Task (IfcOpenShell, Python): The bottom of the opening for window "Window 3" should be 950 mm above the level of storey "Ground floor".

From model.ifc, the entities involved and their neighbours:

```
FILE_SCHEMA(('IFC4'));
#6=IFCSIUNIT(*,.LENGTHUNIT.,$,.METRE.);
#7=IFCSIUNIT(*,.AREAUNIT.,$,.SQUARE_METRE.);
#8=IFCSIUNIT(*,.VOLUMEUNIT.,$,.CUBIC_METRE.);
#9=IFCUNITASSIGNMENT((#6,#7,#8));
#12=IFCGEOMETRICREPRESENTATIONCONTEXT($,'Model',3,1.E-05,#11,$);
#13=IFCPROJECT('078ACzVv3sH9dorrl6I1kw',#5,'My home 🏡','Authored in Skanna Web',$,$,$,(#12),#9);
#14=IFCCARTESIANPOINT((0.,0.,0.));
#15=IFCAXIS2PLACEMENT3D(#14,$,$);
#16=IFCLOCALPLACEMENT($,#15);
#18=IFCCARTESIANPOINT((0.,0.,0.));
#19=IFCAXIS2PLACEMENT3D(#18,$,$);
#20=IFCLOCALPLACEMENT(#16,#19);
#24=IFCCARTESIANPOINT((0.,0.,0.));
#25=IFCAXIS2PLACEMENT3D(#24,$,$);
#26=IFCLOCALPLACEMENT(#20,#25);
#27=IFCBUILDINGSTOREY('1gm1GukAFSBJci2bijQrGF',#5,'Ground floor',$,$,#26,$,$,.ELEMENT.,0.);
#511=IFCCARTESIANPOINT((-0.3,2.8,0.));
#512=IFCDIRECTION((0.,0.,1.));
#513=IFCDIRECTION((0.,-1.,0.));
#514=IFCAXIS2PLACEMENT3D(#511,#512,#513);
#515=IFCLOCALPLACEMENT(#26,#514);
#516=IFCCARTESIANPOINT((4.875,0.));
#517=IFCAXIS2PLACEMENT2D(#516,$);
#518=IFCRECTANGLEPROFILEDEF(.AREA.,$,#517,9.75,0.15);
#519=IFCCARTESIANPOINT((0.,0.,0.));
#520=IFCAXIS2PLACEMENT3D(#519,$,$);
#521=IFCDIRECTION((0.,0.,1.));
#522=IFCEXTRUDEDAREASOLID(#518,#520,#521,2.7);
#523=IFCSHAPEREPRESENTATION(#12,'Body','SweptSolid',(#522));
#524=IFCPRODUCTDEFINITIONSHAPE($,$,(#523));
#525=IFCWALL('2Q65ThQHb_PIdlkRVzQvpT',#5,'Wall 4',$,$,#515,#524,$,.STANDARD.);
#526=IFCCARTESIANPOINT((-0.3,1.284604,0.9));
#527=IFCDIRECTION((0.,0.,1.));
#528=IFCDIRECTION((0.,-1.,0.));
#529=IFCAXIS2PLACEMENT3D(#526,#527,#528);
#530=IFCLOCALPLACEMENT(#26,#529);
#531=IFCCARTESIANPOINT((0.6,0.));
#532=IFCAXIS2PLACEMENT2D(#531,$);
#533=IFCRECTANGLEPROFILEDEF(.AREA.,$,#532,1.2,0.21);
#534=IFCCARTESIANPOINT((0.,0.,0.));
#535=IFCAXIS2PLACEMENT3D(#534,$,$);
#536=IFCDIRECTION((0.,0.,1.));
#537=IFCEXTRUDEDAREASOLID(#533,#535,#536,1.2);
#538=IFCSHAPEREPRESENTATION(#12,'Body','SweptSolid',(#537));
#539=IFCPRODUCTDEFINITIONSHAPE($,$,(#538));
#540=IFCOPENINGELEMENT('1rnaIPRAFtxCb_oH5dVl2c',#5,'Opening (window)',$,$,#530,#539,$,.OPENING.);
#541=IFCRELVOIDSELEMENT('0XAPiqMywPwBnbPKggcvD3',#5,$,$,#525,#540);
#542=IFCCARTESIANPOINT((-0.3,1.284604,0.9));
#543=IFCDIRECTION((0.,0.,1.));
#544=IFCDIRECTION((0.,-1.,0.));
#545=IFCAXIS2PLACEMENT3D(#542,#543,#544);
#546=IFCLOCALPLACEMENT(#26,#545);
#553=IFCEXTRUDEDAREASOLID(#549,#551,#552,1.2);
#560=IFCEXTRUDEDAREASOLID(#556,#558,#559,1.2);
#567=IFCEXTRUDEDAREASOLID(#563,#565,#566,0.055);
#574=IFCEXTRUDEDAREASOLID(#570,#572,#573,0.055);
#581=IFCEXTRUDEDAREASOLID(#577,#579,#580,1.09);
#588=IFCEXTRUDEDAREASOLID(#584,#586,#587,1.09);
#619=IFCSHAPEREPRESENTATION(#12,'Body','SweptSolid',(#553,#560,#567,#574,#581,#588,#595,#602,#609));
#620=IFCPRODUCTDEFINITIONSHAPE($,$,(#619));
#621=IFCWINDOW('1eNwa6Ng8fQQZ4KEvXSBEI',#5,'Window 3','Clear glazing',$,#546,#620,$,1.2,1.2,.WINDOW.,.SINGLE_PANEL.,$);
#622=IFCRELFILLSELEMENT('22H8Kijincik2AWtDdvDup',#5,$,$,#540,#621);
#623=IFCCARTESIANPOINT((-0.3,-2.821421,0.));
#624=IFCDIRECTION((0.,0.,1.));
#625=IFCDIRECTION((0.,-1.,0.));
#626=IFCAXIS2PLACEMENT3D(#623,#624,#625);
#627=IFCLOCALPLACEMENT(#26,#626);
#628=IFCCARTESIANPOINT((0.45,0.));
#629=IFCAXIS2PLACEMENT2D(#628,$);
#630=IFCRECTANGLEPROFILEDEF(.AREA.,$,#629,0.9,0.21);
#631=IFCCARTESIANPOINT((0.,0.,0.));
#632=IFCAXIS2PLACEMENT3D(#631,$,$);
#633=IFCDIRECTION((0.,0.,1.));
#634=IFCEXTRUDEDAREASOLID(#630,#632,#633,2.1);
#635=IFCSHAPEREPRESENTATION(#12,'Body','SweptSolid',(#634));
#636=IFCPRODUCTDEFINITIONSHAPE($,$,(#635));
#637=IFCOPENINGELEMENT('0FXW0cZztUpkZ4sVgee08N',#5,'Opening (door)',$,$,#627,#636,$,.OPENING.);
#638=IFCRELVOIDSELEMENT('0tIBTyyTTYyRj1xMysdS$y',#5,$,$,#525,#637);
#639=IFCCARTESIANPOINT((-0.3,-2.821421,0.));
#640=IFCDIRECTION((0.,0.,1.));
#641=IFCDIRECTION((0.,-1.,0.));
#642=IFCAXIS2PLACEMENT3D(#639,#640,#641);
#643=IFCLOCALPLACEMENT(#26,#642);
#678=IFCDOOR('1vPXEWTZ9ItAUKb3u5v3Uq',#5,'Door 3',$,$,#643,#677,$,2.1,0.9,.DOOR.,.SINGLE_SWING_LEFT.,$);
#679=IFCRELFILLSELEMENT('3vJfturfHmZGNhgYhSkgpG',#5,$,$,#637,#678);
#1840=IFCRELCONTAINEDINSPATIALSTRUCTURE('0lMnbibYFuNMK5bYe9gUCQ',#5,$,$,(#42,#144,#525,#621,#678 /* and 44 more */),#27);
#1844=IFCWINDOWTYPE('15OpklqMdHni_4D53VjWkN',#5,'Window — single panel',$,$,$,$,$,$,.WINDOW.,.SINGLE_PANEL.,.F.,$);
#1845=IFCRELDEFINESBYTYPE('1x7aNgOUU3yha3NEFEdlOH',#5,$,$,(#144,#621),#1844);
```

```python
import numpy as np
import ifcopenshell
import ifcopenshell.api.geometry
import ifcopenshell.geom
import ifcopenshell.util.element
import ifcopenshell.util.placement
import ifcopenshell.util.shape
import ifcopenshell.util.unit

model = ifcopenshell.open("model.ifc")
unit_scale = ifcopenshell.util.unit.calculate_unit_scale(model)

window = model.by_guid("1eNwa6Ng8fQQZ4KEvXSBEI")
opening = window.FillsVoids[0].RelatingOpeningElement
storey = ifcopenshell.util.element.get_container(window, ifc_class="IfcBuildingStorey")
level = ifcopenshell.util.placement.get_local_placement(storey.ObjectPlacement)[2, 3]

# The opening's origin need not be at the sill, so measure its lowest point.
shape = ifcopenshell.geom.create_shape(ifcopenshell.geom.settings(), opening)
bottom = ifcopenshell.util.shape.get_shape_bottom_elevation(shape, shape.geometry) / unit_scale
dz = level + 0.95 - bottom

shift = np.array([0.0, 0.0, dz])
# The window is not placed relative to its opening, so move both.
for product in (opening, window):
    matrix = ifcopenshell.util.placement.get_local_placement(product.ObjectPlacement)
    matrix[:3, 3] += shift
    ifcopenshell.api.geometry.edit_object_placement(model, product=product, matrix=matrix, is_si=False)

print(f"moved by {dz * unit_scale:+.3f} m")

model.write("model-out.ifc")
```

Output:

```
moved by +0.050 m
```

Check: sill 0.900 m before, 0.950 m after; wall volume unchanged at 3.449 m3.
